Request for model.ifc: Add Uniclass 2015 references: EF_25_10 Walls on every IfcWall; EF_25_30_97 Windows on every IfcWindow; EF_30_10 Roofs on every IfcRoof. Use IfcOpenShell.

First a look at what the model holds.

```python
import ifcopenshell

model = ifcopenshell.open("model.ifc")
print(model.schema)
print("classifications:", [c.Name for c in model.by_type("IfcClassification")])
for ifc_class in ("IfcDoor", "IfcRoof", "IfcStair", "IfcWall", "IfcWindow"):
    print(ifc_class, len(model.by_type(ifc_class)))
```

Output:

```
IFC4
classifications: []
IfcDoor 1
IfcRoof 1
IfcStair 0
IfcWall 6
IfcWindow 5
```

```python
import ifcopenshell
import ifcopenshell.api.classification

model = ifcopenshell.open("model.ifc")

system = ifcopenshell.api.classification.add_classification(model, classification="Uniclass 2015")

codes = {
    "IfcWall": ("EF_25_10", "Walls"),
    "IfcWindow": ("EF_25_30_97", "Windows"),
    "IfcRoof": ("EF_30_10", "Roofs"),
}
for ifc_class, (code, name) in codes.items():
    products = model.by_type(ifc_class)
    ifcopenshell.api.classification.add_reference(
        model, products=products, classification=system, identification=code, name=name
    )
    print(code, len(products))

model.write("model_updated.ifc")
```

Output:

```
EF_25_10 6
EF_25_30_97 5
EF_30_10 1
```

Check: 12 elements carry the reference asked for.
